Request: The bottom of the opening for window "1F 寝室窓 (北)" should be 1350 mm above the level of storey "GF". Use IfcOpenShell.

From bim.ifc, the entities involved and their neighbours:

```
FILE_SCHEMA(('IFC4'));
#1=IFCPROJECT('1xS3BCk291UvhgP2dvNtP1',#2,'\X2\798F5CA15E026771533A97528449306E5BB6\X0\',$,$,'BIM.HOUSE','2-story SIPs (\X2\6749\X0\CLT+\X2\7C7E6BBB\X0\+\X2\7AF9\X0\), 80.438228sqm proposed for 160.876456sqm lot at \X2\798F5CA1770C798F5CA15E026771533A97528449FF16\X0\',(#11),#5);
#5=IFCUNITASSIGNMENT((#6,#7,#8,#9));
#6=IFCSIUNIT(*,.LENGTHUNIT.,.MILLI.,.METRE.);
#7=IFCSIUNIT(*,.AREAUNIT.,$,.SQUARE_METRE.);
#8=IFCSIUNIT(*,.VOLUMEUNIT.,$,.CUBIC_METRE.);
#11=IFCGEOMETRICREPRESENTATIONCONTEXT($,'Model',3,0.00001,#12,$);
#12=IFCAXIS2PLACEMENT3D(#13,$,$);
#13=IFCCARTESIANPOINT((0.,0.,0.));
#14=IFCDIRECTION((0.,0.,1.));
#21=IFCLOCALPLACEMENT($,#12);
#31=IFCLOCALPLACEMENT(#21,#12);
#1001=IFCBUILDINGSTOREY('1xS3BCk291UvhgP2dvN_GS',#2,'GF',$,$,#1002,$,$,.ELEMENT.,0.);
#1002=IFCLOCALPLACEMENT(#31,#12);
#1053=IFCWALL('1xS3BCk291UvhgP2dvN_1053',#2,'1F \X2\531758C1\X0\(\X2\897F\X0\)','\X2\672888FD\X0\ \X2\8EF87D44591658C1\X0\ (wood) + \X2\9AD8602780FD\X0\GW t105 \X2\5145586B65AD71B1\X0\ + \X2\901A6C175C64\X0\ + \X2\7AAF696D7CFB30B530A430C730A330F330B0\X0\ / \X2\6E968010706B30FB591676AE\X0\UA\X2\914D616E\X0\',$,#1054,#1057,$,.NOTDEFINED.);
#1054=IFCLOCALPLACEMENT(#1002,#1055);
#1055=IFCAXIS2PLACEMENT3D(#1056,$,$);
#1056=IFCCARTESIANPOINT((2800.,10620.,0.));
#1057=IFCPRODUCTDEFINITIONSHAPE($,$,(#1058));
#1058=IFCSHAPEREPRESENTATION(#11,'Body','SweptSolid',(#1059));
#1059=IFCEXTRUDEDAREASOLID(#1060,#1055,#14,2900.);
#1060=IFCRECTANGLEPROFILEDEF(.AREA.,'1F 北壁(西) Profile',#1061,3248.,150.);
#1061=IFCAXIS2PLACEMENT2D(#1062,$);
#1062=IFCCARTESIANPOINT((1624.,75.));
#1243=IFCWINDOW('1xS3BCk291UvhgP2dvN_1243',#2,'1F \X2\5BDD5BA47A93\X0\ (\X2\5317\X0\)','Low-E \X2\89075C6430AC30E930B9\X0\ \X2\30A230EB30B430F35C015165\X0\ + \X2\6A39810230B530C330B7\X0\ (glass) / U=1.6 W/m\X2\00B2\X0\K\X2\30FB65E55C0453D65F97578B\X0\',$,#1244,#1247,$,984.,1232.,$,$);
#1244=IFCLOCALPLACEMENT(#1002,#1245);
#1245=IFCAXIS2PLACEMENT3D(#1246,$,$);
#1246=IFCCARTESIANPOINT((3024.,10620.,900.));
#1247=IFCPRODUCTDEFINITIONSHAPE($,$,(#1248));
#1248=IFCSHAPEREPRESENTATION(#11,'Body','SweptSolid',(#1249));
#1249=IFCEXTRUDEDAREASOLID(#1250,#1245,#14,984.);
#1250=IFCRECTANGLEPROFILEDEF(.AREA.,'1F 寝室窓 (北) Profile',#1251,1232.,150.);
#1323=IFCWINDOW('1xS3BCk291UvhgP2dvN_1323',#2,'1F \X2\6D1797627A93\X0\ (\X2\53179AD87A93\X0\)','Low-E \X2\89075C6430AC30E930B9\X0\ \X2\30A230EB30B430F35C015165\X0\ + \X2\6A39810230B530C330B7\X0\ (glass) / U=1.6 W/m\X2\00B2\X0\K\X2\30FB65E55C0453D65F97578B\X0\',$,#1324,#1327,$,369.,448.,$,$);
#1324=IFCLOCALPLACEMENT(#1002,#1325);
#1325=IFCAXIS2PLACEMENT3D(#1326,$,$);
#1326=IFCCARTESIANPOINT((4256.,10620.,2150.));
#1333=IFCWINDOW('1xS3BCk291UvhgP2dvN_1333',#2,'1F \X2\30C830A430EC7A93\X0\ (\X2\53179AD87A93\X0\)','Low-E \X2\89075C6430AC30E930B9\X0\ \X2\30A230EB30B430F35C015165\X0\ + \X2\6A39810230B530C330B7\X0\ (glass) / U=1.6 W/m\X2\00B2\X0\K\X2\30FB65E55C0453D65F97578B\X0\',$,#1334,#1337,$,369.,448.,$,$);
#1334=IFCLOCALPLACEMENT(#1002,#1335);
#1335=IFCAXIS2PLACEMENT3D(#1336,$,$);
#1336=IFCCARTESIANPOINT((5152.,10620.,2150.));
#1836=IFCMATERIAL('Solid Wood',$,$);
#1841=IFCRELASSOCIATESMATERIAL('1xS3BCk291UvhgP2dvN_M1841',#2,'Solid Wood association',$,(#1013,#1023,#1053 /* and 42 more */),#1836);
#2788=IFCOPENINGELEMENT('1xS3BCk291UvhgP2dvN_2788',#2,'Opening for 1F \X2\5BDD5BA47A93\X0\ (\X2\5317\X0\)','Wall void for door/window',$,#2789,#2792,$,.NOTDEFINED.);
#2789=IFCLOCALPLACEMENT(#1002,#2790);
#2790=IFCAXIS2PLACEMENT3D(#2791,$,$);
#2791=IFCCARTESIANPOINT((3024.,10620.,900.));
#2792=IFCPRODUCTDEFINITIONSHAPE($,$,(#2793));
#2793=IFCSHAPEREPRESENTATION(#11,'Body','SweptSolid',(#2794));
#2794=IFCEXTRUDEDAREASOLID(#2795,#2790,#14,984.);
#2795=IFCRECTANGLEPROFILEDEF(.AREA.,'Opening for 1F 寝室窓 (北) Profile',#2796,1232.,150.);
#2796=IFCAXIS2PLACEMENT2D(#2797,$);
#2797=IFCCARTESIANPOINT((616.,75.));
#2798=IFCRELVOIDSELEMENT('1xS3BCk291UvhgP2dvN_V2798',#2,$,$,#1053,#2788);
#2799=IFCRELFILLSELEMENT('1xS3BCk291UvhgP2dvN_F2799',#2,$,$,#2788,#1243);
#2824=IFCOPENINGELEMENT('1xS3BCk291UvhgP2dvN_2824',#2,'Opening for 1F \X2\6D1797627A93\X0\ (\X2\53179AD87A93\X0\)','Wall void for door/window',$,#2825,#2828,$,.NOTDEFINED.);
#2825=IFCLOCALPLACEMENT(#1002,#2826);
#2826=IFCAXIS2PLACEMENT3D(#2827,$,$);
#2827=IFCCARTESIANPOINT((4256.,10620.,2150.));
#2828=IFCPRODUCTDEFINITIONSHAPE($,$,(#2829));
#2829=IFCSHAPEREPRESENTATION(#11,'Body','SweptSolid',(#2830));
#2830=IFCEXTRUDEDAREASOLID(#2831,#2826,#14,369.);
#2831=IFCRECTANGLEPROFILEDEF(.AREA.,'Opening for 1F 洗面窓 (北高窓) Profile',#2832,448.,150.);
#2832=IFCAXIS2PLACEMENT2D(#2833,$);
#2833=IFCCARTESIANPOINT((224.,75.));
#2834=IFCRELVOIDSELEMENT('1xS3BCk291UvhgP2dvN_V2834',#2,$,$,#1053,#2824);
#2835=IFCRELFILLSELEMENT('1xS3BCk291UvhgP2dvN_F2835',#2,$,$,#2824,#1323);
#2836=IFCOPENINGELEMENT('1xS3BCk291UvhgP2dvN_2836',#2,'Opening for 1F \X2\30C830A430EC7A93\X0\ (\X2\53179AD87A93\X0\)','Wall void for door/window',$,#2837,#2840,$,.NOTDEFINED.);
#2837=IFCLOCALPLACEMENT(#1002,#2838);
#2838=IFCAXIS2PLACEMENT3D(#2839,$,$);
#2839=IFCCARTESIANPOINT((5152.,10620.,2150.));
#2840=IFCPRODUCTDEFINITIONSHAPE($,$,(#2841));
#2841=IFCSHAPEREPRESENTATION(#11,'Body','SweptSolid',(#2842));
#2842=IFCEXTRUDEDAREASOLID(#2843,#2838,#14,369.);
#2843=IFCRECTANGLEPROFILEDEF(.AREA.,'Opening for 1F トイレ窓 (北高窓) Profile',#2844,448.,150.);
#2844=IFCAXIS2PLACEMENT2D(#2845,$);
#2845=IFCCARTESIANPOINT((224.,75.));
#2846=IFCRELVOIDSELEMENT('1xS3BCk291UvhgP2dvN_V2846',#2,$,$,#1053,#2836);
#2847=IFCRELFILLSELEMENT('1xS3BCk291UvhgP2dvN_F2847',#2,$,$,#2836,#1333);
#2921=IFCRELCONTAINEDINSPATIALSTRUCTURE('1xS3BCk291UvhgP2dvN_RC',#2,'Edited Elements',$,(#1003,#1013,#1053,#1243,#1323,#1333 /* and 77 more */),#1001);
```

```python
import numpy as np
import ifcopenshell
import ifcopenshell.api.geometry
import ifcopenshell.geom
import ifcopenshell.util.element
import ifcopenshell.util.placement
import ifcopenshell.util.shape
import ifcopenshell.util.unit

model = ifcopenshell.open("bim.ifc")
unit_scale = ifcopenshell.util.unit.calculate_unit_scale(model)

window = model.by_guid("1xS3BCk291UvhgP2dvN_1243")
opening = window.FillsVoids[0].RelatingOpeningElement
storey = ifcopenshell.util.element.get_container(window, ifc_class="IfcBuildingStorey")
level = ifcopenshell.util.placement.get_local_placement(storey.ObjectPlacement)[2, 3]

# The opening's origin need not be at the sill, so measure its lowest point.
shape = ifcopenshell.geom.create_shape(ifcopenshell.geom.settings(), opening)
bottom = ifcopenshell.util.shape.get_shape_bottom_elevation(shape, shape.geometry) / unit_scale
dz = level + 1.35 / unit_scale - bottom

shift = np.array([0.0, 0.0, dz])
# The window is not placed relative to its opening, so move both.
for product in (opening, window):
    matrix = ifcopenshell.util.placement.get_local_placement(product.ObjectPlacement)
    matrix[:3, 3] += shift
    ifcopenshell.api.geometry.edit_object_placement(model, product=product, matrix=matrix, is_si=False)

print(f"moved by {dz * unit_scale:+.3f} m")

model.write("bim_v2.ifc")
```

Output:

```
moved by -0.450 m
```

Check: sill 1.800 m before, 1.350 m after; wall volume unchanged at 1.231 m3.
